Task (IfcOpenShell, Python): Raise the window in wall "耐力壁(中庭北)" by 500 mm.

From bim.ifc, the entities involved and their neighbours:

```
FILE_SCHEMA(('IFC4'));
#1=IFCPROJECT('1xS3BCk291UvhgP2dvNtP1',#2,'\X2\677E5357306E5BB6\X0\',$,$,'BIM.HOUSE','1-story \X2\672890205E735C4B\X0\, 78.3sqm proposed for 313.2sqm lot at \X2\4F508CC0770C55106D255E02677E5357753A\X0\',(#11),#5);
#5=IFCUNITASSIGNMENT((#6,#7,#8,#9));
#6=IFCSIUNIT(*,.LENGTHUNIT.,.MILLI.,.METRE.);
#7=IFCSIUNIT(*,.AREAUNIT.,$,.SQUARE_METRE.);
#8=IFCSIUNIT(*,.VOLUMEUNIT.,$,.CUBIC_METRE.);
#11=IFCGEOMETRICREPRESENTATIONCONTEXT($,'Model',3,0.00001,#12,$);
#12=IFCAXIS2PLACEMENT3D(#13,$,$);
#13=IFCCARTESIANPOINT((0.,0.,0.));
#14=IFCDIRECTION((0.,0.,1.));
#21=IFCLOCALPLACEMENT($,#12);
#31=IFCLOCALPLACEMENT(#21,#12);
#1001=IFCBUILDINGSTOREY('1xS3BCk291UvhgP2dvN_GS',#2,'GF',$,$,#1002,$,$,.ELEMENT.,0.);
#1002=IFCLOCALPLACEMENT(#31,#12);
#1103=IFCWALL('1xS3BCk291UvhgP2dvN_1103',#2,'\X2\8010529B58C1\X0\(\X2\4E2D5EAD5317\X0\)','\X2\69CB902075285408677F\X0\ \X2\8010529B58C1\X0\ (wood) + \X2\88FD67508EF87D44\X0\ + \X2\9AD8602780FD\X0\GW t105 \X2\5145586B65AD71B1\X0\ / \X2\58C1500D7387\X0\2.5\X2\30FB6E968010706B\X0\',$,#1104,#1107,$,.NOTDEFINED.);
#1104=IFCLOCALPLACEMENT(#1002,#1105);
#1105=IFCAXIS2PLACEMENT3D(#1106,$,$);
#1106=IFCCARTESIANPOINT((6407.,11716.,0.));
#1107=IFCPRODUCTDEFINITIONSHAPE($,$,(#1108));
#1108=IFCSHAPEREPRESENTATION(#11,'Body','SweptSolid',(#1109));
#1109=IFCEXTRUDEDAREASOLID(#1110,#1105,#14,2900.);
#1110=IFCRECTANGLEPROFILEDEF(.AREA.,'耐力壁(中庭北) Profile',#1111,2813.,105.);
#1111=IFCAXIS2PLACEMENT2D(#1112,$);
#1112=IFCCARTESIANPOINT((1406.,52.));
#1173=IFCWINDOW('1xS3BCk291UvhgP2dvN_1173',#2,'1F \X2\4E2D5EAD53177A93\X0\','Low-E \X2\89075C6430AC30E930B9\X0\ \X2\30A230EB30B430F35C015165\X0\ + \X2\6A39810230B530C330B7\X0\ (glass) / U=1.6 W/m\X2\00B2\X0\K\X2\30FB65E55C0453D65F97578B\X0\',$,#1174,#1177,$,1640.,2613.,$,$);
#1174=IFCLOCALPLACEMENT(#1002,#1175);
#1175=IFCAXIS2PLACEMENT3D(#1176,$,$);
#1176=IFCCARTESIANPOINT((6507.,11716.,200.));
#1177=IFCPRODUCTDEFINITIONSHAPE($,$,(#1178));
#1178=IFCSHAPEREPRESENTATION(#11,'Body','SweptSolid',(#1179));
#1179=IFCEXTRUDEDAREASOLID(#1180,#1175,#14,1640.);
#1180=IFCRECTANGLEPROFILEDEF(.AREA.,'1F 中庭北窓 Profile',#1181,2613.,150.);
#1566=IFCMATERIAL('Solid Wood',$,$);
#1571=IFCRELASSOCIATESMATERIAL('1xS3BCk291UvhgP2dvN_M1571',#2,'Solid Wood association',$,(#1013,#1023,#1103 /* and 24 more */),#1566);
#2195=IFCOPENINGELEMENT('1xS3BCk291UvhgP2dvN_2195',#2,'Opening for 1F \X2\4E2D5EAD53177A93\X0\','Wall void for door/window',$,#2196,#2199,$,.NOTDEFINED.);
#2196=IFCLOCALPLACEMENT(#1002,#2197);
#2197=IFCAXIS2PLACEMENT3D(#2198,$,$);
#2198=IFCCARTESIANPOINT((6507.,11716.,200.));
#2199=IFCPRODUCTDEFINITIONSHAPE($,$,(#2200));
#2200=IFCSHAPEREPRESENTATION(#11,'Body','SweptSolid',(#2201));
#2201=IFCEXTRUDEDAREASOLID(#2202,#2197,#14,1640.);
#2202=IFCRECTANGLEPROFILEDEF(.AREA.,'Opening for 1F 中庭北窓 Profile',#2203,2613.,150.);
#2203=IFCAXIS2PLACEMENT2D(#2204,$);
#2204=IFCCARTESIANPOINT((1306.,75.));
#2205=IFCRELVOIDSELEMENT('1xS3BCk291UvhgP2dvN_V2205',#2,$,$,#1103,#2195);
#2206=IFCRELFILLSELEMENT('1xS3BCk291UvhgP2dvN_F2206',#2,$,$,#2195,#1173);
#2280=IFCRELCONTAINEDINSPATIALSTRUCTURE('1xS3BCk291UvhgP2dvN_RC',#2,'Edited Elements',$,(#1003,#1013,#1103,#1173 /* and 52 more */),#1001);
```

```python
import numpy as np
import ifcopenshell
import ifcopenshell.api.geometry
import ifcopenshell.util.placement
import ifcopenshell.util.unit

model = ifcopenshell.open("bim.ifc")
unit_scale = ifcopenshell.util.unit.calculate_unit_scale(model)

window = model.by_guid("1xS3BCk291UvhgP2dvN_1173")
opening = window.FillsVoids[0].RelatingOpeningElement
dz = 0.5 / unit_scale

shift = np.array([0.0, 0.0, dz])
# The window is not placed relative to its opening, so move both.
for product in (opening, window):
    matrix = ifcopenshell.util.placement.get_local_placement(product.ObjectPlacement)
    matrix[:3, 3] += shift
    ifcopenshell.api.geometry.edit_object_placement(model, product=product, matrix=matrix, is_si=False)

print(f"moved by {dz * unit_scale:+.3f} m")

model.write("bim-out.ifc")
```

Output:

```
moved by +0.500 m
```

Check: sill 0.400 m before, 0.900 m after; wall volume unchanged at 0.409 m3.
